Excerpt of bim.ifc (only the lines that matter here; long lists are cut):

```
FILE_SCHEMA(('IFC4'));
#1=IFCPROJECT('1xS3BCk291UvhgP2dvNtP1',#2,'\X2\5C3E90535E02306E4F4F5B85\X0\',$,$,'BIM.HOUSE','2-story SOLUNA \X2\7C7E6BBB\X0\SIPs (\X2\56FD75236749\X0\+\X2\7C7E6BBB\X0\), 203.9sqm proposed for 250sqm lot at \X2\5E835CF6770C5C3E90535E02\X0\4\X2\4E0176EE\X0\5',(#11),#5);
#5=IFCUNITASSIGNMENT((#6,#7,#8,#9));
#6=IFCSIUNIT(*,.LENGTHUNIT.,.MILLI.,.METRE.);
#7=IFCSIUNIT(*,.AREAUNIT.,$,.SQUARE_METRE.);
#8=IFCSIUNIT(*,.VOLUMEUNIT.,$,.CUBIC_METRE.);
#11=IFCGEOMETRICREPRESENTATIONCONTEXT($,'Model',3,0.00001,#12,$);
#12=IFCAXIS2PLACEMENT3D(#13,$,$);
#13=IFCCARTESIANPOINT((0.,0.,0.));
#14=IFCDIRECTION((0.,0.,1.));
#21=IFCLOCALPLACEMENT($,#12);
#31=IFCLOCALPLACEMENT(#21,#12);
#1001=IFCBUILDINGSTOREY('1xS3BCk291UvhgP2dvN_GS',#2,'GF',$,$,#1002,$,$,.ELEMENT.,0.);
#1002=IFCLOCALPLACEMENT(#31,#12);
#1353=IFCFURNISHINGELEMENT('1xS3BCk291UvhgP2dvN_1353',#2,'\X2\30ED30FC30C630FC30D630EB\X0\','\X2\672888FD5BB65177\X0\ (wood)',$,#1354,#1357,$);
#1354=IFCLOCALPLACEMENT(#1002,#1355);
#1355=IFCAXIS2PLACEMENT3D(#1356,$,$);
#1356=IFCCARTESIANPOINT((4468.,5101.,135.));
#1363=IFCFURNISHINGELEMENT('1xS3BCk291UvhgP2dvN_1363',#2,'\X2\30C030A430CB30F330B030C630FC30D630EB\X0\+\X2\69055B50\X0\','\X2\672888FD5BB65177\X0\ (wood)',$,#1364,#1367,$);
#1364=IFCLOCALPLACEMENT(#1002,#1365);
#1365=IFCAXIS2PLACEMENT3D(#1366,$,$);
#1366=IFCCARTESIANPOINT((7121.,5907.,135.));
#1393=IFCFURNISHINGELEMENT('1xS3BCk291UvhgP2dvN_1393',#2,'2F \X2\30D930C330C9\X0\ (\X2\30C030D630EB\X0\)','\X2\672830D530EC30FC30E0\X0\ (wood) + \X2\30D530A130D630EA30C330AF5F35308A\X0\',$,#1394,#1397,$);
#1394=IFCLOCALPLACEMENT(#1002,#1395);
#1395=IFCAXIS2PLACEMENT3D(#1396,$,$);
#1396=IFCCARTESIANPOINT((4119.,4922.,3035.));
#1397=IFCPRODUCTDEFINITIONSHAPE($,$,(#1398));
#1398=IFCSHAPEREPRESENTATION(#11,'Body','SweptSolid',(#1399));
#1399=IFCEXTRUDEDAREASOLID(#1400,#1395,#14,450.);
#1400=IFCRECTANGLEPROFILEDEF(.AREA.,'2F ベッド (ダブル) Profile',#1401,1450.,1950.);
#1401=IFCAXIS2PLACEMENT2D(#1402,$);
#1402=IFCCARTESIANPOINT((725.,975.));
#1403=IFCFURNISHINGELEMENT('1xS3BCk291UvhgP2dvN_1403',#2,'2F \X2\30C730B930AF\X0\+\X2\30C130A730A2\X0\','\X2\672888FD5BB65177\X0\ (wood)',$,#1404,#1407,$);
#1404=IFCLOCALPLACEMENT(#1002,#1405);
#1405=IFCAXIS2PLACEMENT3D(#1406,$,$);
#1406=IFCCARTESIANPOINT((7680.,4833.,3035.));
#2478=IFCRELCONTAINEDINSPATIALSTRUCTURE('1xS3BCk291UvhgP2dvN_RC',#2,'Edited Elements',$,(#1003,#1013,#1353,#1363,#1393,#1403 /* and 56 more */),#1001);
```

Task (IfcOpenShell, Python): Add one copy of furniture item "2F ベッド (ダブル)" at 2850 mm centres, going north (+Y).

```python
import numpy as np
import ifcopenshell
import ifcopenshell.api.geometry
import ifcopenshell.api.root
import ifcopenshell.util.element
import ifcopenshell.util.placement
import ifcopenshell.util.unit

model = ifcopenshell.open("bim.ifc")
unit_scale = ifcopenshell.util.unit.calculate_unit_scale(model)


def reuse_history(source, copy):
    """copy_class also copies each property set's owner history, people and application; keep the originals."""
    for rel in copy.IsDefinedBy:
        if rel.is_a("IfcRelDefinesByProperties") and (history := rel.RelatingPropertyDefinition.OwnerHistory):
            rel.RelatingPropertyDefinition.OwnerHistory = source.OwnerHistory
            ifcopenshell.util.element.remove_deep2(model, history)


source = model.by_guid("1xS3BCk291UvhgP2dvN_1393")
base = ifcopenshell.util.placement.get_local_placement(source.ObjectPlacement)
step = np.array([0.0, 1.0, 0.0]) * 2.85 / unit_scale

for i in range(1, 2):
    copy = ifcopenshell.api.root.copy_class(model, product=source)
    copy.Representation = ifcopenshell.util.element.copy_deep(
        model, source.Representation, exclude=["IfcGeometricRepresentationContext", "IfcRepresentationMap"]
    )
    reuse_history(source, copy)
    matrix = base.copy()
    matrix[:3, 3] += i * step
    print("added at", matrix[:3, 3].round(3) + 0.0)
    ifcopenshell.api.geometry.edit_object_placement(model, product=copy, matrix=matrix, is_si=False)

model.write("bim_rev.ifc")
```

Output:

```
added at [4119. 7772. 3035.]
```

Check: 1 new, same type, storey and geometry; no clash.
